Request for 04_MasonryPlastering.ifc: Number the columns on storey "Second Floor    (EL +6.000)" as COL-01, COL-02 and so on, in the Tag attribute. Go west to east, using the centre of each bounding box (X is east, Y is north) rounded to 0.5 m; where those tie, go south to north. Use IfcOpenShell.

First a look at what the model holds.

```python
import ifcopenshell
import ifcopenshell.util.element
import ifcopenshell.util.placement

model = ifcopenshell.open("04_MasonryPlastering.ifc")
print(model.schema)
storey = next(s for s in model.by_type("IfcBuildingStorey") if s.Name == "Second Floor    (EL +6.000)")
columns = [e for e in ifcopenshell.util.element.get_decomposition(storey) if e.is_a("IfcColumn")]
for e in sorted(columns, key=lambda e: e.id()):
    origin = ifcopenshell.util.placement.get_local_placement(e.ObjectPlacement)[:3, 3]
    print(e.id(), e.Tag, e.Name, origin.round(2) + 0.0, sep=" | ")
```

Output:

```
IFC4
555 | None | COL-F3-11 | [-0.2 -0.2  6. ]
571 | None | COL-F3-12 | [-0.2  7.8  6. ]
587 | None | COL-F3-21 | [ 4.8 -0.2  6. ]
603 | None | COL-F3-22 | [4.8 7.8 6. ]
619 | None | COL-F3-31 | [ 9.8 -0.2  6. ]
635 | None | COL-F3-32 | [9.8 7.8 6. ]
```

```python
import ifcopenshell
import ifcopenshell.geom
import ifcopenshell.util.element
import ifcopenshell.util.shape

model = ifcopenshell.open("04_MasonryPlastering.ifc")
settings = ifcopenshell.geom.settings()
settings.set("use-world-coords", True)


def centre(element):
    shape = ifcopenshell.geom.create_shape(settings, element)
    return ifcopenshell.util.shape.get_bbox_centroid(shape.geometry)


storey = next(s for s in model.by_type("IfcBuildingStorey") if s.Name == "Second Floor    (EL +6.000)")
columns = [e for e in ifcopenshell.util.element.get_decomposition(storey) if e.is_a("IfcColumn")]

# Insertion points can sit at a corner or the storey origin, so sort by the geometry (in metres).
centres = {e: centre(e) for e in columns}
columns.sort(key=lambda e: (round(centres[e][0] / 0.5), centres[e][1]))

for i, e in enumerate(columns, start=1):
    number = f"COL-{i:02d}"
    e.Tag = number
    print(e.id(), number)

model.write("04_MasonryPlastering_v2.ifc")
```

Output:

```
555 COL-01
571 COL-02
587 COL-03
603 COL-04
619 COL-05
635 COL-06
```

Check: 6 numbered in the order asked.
